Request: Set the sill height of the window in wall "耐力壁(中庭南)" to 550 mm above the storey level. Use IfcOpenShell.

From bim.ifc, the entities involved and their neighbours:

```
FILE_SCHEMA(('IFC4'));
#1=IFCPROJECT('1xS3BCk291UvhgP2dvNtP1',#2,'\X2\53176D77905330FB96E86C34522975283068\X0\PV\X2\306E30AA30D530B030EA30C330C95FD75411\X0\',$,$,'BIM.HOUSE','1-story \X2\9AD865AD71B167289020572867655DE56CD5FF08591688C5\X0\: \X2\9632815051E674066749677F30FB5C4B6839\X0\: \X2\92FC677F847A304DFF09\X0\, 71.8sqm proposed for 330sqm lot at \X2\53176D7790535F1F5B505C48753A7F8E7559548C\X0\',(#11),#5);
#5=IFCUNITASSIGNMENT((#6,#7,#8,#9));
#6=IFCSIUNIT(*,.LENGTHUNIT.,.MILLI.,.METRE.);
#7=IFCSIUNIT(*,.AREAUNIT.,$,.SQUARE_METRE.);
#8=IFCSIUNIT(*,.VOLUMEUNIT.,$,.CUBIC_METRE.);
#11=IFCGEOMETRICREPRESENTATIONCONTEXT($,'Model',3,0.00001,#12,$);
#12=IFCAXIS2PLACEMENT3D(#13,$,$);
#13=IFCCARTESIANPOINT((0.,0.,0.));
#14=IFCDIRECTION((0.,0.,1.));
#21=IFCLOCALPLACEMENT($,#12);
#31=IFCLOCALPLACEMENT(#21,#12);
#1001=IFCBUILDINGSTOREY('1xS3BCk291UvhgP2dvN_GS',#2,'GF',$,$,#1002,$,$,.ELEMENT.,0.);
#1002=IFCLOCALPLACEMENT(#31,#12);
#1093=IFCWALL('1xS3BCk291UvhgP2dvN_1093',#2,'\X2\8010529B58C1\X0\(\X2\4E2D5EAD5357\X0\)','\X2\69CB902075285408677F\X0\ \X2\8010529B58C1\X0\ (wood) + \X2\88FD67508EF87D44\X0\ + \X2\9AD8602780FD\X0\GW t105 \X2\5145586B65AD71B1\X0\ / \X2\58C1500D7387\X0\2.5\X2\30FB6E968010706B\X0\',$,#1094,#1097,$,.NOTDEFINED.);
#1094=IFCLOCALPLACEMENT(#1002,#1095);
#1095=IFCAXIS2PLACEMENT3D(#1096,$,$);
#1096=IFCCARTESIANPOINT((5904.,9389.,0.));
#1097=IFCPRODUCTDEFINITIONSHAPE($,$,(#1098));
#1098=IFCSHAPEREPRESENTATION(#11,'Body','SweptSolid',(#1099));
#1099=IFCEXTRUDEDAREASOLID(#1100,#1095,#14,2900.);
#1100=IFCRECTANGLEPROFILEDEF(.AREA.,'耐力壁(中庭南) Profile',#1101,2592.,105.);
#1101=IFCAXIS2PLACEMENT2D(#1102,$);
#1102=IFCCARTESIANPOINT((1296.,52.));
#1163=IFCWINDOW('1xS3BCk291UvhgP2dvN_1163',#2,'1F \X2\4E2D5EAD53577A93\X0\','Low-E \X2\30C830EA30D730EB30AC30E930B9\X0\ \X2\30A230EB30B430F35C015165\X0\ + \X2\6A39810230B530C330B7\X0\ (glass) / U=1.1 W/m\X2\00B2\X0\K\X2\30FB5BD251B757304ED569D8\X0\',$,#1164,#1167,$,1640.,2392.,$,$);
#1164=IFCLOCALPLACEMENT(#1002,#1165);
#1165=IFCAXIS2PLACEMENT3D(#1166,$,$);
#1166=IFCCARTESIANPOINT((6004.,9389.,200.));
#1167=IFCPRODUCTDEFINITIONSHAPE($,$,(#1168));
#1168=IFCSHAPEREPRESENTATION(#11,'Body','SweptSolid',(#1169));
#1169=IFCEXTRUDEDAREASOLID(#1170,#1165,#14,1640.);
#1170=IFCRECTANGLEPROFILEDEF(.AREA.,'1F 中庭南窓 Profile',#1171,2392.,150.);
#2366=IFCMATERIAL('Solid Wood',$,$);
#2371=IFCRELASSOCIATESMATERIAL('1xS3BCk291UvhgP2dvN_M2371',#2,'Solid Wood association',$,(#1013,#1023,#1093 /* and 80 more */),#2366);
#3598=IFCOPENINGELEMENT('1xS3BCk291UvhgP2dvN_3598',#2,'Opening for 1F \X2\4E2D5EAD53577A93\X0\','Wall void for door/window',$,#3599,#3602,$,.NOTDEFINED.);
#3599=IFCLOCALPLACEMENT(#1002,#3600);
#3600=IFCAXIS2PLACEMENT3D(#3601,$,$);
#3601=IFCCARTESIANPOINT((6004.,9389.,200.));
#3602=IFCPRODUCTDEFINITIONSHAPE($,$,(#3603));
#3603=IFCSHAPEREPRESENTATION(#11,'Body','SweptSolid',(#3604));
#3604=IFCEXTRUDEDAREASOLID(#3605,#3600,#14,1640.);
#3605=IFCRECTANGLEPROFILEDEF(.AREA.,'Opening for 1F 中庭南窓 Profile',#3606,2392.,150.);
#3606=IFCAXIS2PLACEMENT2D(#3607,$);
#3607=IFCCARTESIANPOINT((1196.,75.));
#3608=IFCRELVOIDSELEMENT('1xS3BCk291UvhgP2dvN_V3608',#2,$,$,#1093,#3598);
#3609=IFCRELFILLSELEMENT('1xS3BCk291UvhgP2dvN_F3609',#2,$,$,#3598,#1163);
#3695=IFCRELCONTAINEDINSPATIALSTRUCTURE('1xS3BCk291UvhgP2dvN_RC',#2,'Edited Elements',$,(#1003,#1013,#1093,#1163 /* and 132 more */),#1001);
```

```python
import numpy as np
import ifcopenshell
import ifcopenshell.api.geometry
import ifcopenshell.geom
import ifcopenshell.util.element
import ifcopenshell.util.placement
import ifcopenshell.util.shape
import ifcopenshell.util.unit

model = ifcopenshell.open("bim.ifc")
unit_scale = ifcopenshell.util.unit.calculate_unit_scale(model)

window = model.by_guid("1xS3BCk291UvhgP2dvN_1163")
opening = window.FillsVoids[0].RelatingOpeningElement
storey = ifcopenshell.util.element.get_container(window, ifc_class="IfcBuildingStorey")
level = ifcopenshell.util.placement.get_local_placement(storey.ObjectPlacement)[2, 3]

# The opening's origin need not be at the sill, so measure its lowest point.
shape = ifcopenshell.geom.create_shape(ifcopenshell.geom.settings(), opening)
bottom = ifcopenshell.util.shape.get_shape_bottom_elevation(shape, shape.geometry) / unit_scale
dz = level + 550.0 - bottom

shift = np.array([0.0, 0.0, dz])
# The window is not placed relative to its opening, so move both.
for product in (opening, window):
    matrix = ifcopenshell.util.placement.get_local_placement(product.ObjectPlacement)
    matrix[:3, 3] += shift
    ifcopenshell.api.geometry.edit_object_placement(model, product=product, matrix=matrix, is_si=False)

print(f"moved by {dz * unit_scale:+.3f} m")

model.write("bim_rev.ifc")
```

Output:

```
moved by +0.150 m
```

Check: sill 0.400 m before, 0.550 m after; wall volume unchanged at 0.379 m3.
